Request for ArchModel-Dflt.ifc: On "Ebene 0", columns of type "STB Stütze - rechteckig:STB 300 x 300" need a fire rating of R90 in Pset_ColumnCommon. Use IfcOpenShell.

First a look at what the model holds.

```python
import ifcopenshell
import ifcopenshell.util.element

model = ifcopenshell.open("ArchModel-Dflt.ifc")
print(model.schema)
storey = next(s for s in model.by_type("IfcBuildingStorey") if s.Name == "Ebene 0")
columns = [e for e in ifcopenshell.util.element.get_decomposition(storey) if e.is_a("IfcColumn")]
seen = {}
for e in columns:
    element_type = ifcopenshell.util.element.get_type(e)
    key = (element_type.Name if element_type != e and element_type else None, ifcopenshell.util.element.get_pset(e, "Pset_ColumnCommon", "FireRating"))
    seen[key] = seen.get(key, 0) + 1
for (name, value), count in sorted(seen.items(), key=str):
    print(count, "x", name, "|", value)
```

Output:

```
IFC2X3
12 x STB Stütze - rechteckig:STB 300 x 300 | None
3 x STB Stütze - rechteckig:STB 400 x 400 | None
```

```python
import ifcopenshell
import ifcopenshell.api.pset
import ifcopenshell.util.element

model = ifcopenshell.open("ArchModel-Dflt.ifc")

storey = next(s for s in model.by_type("IfcBuildingStorey") if s.Name == "Ebene 0")
columns = [e for e in ifcopenshell.util.element.get_decomposition(storey) if e.is_a("IfcColumn")]

count = 0
for e in columns:
    element_type = ifcopenshell.util.element.get_type(e)
    if element_type in (None, e) or element_type.Name != "STB Stütze - rechteckig:STB 300 x 300":
        continue
    # add_pset returns the element's existing set when there is one.
    pset = ifcopenshell.api.pset.add_pset(model, product=e, name="Pset_ColumnCommon")
    ifcopenshell.api.pset.edit_pset(model, pset=pset, properties={"FireRating": "R90"})
    count += 1

print(count, "columns updated")

model.write("ArchModel-Dflt_edited.ifc")
```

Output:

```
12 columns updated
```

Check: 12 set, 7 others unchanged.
